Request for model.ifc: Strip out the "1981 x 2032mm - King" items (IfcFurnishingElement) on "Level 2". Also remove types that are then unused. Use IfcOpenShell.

First a look at what the model holds.

```python
import ifcopenshell
import ifcopenshell.util.element

model = ifcopenshell.open("model.ifc")
print(model.schema)
storey = next(s for s in model.by_type("IfcBuildingStorey") if s.Name == "Level 2")
furniture = [e for e in ifcopenshell.util.element.get_decomposition(storey) if e.is_a("IfcFurnishingElement")]
seen = {}
for e in furniture:
    element_type = ifcopenshell.util.element.get_type(e)
    name = element_type.Name if element_type not in (None, e) else None
    seen[name] = seen.get(name, 0) + 1
for name, count in sorted(seen.items(), key=str):
    print(count, "x", name)
```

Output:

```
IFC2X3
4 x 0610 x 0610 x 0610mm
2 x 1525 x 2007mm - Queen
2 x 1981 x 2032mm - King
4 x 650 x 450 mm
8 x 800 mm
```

```python
import ifcopenshell
import ifcopenshell.api.root
import ifcopenshell.util.element

model = ifcopenshell.open("model.ifc")

storey = next(s for s in model.by_type("IfcBuildingStorey") if s.Name == "Level 2")
furniture = [e for e in ifcopenshell.util.element.get_decomposition(storey) if e.is_a("IfcFurnishingElement")]
targets = [e for e in furniture if (t := ifcopenshell.util.element.get_type(e)) not in (None, e) and t.Name == "1981 x 2032mm - King"]
types = {ifcopenshell.util.element.get_type(e) for e in targets} - {None, *targets}

for e in targets:
    ifcopenshell.api.root.remove_product(model, product=e)
print(len(targets), "removed")

unused = [t for t in types if not ifcopenshell.util.element.get_types(t)]
for t in unused:
    ifcopenshell.api.root.remove_product(model, product=t)
print(len(unused), "unused types removed")

model.write("model_edited.ifc")
```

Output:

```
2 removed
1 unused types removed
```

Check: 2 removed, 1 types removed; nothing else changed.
